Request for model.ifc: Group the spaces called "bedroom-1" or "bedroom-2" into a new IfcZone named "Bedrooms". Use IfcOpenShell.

First a look at what the model holds.

```python
import ifcopenshell

model = ifcopenshell.open("model.ifc")
print(model.schema)
seen = {}
for space in model.by_type("IfcSpace"):
    seen[space.Name] = seen.get(space.Name, 0) + 1
for name, count in sorted(seen.items(), key=str):
    print(count, "x", name)
print("zones:", [z.Name for z in model.by_type("IfcZone")][:20])
```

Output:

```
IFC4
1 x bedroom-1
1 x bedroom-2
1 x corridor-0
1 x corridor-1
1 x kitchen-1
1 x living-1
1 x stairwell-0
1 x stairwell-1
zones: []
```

```python
import ifcopenshell
import ifcopenshell.api.group
import ifcopenshell.api.root

model = ifcopenshell.open("model.ifc")

names = {"bedroom-1", "bedroom-2"}
spaces = [s for s in model.by_type("IfcSpace") if s.Name in names]

zone = ifcopenshell.api.root.create_entity(model, ifc_class="IfcZone", name="Bedrooms")
ifcopenshell.api.group.assign_group(model, products=spaces, group=zone)
print(len(spaces), "spaces in", zone.Name)

model.write("model-out.ifc")
```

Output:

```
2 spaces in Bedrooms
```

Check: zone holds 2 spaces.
